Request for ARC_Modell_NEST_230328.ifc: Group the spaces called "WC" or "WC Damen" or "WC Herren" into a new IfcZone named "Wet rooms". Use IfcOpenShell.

First a look at what the model holds.

```python
import ifcopenshell

model = ifcopenshell.open("ARC_Modell_NEST_230328.ifc")
print(model.schema)
seen = {}
for space in model.by_type("IfcSpace"):
    seen[space.LongName] = seen.get(space.LongName, 0) + 1
for name, count in sorted(seen.items(), key=str):
    print(count, "x", name)
print("zones:", [z.Name for z in model.by_type("IfcZone")][:20])
```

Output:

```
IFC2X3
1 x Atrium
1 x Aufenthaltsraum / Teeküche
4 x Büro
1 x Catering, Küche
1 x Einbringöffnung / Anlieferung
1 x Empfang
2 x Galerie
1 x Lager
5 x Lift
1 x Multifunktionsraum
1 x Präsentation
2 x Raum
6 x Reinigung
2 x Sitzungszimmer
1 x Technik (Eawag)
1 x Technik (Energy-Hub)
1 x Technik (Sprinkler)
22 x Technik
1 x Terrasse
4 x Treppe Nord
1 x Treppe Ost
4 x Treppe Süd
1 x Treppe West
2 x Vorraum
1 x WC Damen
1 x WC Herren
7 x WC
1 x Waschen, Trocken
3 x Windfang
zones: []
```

```python
import ifcopenshell
import ifcopenshell.api.group
import ifcopenshell.api.root

model = ifcopenshell.open("ARC_Modell_NEST_230328.ifc")

names = {"WC", "WC Damen", "WC Herren"}
spaces = [s for s in model.by_type("IfcSpace") if s.LongName in names]

zone = ifcopenshell.api.root.create_entity(model, ifc_class="IfcZone", name="Wet rooms")
ifcopenshell.api.group.assign_group(model, products=spaces, group=zone)
print(len(spaces), "spaces in", zone.Name)

model.write("ARC_Modell_NEST_230328-out.ifc")
```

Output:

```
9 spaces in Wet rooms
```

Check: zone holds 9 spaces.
